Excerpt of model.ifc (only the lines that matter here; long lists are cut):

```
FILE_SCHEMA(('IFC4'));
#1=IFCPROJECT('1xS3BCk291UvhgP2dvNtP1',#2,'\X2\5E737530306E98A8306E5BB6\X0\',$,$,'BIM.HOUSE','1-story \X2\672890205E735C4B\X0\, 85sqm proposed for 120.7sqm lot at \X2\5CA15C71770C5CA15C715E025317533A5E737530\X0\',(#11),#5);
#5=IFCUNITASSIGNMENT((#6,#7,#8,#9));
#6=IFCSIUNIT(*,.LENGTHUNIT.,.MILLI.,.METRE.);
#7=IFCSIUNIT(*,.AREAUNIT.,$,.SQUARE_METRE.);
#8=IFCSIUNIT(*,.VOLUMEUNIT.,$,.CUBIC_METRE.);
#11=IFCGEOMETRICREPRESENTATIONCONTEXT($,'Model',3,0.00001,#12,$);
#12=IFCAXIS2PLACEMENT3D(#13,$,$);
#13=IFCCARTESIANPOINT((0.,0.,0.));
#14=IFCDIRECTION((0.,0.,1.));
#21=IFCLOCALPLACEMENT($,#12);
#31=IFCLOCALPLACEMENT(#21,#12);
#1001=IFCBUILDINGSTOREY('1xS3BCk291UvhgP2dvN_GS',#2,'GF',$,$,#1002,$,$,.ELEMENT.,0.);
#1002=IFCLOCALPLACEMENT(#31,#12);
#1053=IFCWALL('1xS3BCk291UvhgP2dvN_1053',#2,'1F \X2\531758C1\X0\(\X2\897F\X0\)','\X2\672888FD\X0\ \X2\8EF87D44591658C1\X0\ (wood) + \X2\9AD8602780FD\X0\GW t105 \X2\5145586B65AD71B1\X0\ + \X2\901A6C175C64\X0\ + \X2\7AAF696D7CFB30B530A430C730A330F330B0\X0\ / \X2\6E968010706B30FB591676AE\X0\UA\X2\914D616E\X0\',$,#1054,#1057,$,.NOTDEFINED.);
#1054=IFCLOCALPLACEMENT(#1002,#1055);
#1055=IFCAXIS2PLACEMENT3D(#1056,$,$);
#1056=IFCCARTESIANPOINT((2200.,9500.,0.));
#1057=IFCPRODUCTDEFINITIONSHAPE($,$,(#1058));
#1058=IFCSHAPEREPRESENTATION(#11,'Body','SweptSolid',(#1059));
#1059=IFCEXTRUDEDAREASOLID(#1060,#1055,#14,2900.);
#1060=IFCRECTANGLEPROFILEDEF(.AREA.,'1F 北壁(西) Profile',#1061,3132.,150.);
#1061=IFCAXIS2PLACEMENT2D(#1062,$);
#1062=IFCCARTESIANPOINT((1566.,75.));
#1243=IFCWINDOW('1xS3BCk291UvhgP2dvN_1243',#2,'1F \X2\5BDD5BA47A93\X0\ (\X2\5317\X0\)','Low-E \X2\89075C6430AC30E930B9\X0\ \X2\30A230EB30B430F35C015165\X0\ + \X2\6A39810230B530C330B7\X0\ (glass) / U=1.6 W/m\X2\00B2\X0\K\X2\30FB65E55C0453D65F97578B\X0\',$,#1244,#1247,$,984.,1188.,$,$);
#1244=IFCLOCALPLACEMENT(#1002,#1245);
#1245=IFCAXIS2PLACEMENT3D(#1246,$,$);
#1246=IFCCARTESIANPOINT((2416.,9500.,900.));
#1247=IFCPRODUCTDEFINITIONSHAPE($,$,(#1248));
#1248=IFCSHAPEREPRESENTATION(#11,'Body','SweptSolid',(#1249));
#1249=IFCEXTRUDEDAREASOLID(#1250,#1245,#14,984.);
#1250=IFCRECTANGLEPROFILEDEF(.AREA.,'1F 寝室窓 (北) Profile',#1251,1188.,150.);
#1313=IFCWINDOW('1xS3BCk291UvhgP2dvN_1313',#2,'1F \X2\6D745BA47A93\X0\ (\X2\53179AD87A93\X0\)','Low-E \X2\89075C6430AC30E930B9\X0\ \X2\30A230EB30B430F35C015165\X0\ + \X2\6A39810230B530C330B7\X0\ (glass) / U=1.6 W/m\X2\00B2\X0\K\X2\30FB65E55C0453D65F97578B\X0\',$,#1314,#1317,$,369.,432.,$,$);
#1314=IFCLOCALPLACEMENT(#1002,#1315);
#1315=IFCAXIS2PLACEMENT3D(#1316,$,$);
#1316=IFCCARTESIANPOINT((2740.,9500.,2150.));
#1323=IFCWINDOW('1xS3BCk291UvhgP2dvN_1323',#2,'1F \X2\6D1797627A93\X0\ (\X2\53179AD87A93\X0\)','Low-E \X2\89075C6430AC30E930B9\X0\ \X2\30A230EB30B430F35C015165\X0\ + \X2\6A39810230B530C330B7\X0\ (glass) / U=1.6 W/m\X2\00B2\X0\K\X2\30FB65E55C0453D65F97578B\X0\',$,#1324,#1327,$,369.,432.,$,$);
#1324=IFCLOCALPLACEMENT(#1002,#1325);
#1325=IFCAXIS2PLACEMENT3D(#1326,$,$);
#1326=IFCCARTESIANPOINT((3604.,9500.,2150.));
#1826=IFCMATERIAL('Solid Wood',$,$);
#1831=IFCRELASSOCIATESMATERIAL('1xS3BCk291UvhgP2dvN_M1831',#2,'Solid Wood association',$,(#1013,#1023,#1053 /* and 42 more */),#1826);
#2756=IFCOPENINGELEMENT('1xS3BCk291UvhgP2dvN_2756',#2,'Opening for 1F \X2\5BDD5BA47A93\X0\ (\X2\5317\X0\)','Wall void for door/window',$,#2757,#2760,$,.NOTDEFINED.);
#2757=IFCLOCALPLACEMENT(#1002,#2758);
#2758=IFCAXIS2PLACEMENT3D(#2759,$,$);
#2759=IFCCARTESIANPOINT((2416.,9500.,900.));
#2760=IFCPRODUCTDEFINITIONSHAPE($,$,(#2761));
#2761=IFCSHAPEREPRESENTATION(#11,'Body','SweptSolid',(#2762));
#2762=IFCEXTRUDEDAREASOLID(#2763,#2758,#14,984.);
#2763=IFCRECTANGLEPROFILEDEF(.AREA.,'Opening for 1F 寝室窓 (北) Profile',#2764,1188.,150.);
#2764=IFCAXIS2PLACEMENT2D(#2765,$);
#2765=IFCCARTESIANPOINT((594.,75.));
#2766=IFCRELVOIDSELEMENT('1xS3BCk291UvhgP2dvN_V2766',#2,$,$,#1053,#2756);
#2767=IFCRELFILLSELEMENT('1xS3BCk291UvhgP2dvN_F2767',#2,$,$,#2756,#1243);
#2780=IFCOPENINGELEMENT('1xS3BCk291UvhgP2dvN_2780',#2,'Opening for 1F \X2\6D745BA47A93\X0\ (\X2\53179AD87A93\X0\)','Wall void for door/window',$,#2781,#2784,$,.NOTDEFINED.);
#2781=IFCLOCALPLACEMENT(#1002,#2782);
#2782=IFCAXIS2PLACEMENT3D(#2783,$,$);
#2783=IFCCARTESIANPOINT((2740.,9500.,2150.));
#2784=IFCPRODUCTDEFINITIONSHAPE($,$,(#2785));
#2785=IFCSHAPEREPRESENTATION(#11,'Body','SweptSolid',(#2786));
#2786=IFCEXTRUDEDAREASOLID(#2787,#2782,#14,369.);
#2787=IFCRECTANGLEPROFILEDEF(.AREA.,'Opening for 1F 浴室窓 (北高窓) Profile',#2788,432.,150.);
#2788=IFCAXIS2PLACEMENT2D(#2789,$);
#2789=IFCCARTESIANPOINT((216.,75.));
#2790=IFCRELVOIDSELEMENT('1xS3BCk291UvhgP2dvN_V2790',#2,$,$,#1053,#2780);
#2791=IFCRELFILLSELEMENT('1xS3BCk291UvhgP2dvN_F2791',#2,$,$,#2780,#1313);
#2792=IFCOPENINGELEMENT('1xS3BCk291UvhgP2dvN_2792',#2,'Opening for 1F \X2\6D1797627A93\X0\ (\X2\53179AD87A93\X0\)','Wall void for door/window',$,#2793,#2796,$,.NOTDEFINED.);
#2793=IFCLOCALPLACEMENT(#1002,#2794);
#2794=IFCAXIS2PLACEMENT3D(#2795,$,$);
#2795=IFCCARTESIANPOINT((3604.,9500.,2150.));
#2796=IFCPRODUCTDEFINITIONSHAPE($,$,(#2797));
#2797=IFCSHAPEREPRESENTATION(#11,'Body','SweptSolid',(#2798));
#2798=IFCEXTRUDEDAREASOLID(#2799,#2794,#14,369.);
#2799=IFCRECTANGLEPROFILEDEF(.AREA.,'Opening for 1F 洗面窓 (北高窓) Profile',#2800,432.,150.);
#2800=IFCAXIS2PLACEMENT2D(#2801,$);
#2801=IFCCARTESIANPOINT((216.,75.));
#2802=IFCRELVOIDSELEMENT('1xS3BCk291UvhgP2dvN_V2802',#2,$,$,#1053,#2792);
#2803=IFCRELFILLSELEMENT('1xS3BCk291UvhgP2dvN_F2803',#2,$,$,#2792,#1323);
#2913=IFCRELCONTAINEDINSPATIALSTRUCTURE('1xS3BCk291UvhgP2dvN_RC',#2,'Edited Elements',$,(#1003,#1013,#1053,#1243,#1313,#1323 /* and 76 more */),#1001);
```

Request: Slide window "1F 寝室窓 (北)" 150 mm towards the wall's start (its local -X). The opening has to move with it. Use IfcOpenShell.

```python
import ifcopenshell
import ifcopenshell.api.geometry
import ifcopenshell.util.placement
import ifcopenshell.util.unit

model = ifcopenshell.open("model.ifc")
unit_scale = ifcopenshell.util.unit.calculate_unit_scale(model)

window = model.by_guid("1xS3BCk291UvhgP2dvN_1243")
opening = window.FillsVoids[0].RelatingOpeningElement
wall = opening.VoidsElements[0].RelatingBuildingElement

wall_matrix = ifcopenshell.util.placement.get_local_placement(wall.ObjectPlacement)
shift = wall_matrix[:3, 0] * -0.15 / unit_scale
before = ifcopenshell.util.placement.get_local_placement(window.ObjectPlacement)[:3, 3].copy()

# The window is not placed relative to its opening, so move both.
for product in (opening, window):
    matrix = ifcopenshell.util.placement.get_local_placement(product.ObjectPlacement)
    matrix[:3, 3] += shift
    ifcopenshell.api.geometry.edit_object_placement(model, product=product, matrix=matrix, is_si=False)

after = ifcopenshell.util.placement.get_local_placement(window.ObjectPlacement)[:3, 3]
print("window moved by", (after - before).round(3) + 0.0)

model.write("model-out.ifc")
```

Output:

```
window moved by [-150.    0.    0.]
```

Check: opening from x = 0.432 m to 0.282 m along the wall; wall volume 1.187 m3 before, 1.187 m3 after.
